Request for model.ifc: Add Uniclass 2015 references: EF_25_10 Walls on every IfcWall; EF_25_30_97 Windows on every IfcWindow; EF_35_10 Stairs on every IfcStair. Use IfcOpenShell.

First a look at what the model holds.

```python
import ifcopenshell

model = ifcopenshell.open("model.ifc")
print(model.schema)
print("classifications:", [c.Name for c in model.by_type("IfcClassification")])
for ifc_class in ("IfcDoor", "IfcRoof", "IfcStair", "IfcWall", "IfcWindow"):
    print(ifc_class, len(model.by_type(ifc_class)))
```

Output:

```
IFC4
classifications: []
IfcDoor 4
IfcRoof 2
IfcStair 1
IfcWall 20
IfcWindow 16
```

```python
import ifcopenshell
import ifcopenshell.api.classification

model = ifcopenshell.open("model.ifc")

system = ifcopenshell.api.classification.add_classification(model, classification="Uniclass 2015")

codes = {
    "IfcWall": ("EF_25_10", "Walls"),
    "IfcWindow": ("EF_25_30_97", "Windows"),
    "IfcStair": ("EF_35_10", "Stairs"),
}
for ifc_class, (code, name) in codes.items():
    products = model.by_type(ifc_class)
    ifcopenshell.api.classification.add_reference(
        model, products=products, classification=system, identification=code, name=name
    )
    print(code, len(products))

model.write("model_v2.ifc")
```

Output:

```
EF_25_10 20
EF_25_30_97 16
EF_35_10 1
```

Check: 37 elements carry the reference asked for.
